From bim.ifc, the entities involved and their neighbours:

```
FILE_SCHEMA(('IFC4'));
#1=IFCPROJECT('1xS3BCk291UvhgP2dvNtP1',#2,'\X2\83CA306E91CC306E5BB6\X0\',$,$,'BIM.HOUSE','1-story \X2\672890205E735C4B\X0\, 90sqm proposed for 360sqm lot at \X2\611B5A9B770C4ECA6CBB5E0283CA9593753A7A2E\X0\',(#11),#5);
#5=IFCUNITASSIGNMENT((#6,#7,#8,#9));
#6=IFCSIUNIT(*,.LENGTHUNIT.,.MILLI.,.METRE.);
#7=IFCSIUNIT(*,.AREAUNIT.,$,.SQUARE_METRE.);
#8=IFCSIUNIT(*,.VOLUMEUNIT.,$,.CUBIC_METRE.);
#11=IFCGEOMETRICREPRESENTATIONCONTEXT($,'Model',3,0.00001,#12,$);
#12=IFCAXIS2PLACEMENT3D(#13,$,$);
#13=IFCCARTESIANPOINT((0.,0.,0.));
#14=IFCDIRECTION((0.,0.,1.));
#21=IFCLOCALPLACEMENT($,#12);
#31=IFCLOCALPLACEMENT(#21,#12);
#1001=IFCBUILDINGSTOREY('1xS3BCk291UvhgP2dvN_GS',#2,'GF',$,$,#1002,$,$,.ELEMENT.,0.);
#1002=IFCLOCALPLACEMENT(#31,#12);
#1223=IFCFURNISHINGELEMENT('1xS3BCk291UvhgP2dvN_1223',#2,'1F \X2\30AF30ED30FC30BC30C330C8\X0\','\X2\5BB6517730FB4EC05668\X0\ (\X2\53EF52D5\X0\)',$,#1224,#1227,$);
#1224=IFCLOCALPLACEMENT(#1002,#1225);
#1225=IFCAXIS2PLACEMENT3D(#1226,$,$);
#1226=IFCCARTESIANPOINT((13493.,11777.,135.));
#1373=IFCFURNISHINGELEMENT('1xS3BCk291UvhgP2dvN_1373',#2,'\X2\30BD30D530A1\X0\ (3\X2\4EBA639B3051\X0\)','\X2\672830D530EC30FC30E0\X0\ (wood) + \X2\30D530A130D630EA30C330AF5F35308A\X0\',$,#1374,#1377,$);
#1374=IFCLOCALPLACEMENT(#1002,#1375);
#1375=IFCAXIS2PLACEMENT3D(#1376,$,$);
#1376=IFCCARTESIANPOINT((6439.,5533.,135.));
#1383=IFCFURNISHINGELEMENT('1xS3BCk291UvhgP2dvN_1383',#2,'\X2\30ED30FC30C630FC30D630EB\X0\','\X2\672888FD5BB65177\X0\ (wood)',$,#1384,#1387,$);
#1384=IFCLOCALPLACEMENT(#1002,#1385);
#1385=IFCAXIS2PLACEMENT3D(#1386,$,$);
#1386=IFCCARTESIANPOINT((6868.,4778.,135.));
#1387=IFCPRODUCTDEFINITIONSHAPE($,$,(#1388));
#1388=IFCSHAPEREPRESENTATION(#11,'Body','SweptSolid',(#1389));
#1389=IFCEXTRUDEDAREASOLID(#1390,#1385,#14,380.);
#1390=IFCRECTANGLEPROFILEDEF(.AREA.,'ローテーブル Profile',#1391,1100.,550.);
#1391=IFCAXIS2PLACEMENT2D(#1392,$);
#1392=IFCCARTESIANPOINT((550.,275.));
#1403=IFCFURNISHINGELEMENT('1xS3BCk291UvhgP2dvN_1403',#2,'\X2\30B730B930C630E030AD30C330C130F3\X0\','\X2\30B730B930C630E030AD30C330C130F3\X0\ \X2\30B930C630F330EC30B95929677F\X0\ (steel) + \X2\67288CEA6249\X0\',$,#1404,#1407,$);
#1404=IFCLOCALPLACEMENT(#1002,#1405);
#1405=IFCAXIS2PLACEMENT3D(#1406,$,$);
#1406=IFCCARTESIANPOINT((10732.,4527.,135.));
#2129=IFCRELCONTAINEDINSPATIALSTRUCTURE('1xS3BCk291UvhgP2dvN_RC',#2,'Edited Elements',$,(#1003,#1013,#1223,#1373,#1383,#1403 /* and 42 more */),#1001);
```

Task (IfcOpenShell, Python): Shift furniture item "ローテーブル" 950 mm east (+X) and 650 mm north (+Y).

```python
import ifcopenshell
import ifcopenshell.api.geometry
import ifcopenshell.util.placement
import ifcopenshell.util.unit

model = ifcopenshell.open("bim.ifc")
unit_scale = ifcopenshell.util.unit.calculate_unit_scale(model)

item = model.by_guid("1xS3BCk291UvhgP2dvN_1383")
matrix = ifcopenshell.util.placement.get_local_placement(item.ObjectPlacement)
matrix[0, 3] += 0.95 / unit_scale
matrix[1, 3] += 0.65 / unit_scale
ifcopenshell.api.geometry.edit_object_placement(model, product=item, matrix=matrix, is_si=False)

print(ifcopenshell.util.placement.get_local_placement(item.ObjectPlacement).round(3) + 0.0)

model.write("bim_v2.ifc")
```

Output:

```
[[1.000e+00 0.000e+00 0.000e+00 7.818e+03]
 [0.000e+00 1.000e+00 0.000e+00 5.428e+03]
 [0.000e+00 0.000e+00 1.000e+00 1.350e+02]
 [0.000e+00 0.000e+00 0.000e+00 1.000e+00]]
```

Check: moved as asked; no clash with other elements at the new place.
